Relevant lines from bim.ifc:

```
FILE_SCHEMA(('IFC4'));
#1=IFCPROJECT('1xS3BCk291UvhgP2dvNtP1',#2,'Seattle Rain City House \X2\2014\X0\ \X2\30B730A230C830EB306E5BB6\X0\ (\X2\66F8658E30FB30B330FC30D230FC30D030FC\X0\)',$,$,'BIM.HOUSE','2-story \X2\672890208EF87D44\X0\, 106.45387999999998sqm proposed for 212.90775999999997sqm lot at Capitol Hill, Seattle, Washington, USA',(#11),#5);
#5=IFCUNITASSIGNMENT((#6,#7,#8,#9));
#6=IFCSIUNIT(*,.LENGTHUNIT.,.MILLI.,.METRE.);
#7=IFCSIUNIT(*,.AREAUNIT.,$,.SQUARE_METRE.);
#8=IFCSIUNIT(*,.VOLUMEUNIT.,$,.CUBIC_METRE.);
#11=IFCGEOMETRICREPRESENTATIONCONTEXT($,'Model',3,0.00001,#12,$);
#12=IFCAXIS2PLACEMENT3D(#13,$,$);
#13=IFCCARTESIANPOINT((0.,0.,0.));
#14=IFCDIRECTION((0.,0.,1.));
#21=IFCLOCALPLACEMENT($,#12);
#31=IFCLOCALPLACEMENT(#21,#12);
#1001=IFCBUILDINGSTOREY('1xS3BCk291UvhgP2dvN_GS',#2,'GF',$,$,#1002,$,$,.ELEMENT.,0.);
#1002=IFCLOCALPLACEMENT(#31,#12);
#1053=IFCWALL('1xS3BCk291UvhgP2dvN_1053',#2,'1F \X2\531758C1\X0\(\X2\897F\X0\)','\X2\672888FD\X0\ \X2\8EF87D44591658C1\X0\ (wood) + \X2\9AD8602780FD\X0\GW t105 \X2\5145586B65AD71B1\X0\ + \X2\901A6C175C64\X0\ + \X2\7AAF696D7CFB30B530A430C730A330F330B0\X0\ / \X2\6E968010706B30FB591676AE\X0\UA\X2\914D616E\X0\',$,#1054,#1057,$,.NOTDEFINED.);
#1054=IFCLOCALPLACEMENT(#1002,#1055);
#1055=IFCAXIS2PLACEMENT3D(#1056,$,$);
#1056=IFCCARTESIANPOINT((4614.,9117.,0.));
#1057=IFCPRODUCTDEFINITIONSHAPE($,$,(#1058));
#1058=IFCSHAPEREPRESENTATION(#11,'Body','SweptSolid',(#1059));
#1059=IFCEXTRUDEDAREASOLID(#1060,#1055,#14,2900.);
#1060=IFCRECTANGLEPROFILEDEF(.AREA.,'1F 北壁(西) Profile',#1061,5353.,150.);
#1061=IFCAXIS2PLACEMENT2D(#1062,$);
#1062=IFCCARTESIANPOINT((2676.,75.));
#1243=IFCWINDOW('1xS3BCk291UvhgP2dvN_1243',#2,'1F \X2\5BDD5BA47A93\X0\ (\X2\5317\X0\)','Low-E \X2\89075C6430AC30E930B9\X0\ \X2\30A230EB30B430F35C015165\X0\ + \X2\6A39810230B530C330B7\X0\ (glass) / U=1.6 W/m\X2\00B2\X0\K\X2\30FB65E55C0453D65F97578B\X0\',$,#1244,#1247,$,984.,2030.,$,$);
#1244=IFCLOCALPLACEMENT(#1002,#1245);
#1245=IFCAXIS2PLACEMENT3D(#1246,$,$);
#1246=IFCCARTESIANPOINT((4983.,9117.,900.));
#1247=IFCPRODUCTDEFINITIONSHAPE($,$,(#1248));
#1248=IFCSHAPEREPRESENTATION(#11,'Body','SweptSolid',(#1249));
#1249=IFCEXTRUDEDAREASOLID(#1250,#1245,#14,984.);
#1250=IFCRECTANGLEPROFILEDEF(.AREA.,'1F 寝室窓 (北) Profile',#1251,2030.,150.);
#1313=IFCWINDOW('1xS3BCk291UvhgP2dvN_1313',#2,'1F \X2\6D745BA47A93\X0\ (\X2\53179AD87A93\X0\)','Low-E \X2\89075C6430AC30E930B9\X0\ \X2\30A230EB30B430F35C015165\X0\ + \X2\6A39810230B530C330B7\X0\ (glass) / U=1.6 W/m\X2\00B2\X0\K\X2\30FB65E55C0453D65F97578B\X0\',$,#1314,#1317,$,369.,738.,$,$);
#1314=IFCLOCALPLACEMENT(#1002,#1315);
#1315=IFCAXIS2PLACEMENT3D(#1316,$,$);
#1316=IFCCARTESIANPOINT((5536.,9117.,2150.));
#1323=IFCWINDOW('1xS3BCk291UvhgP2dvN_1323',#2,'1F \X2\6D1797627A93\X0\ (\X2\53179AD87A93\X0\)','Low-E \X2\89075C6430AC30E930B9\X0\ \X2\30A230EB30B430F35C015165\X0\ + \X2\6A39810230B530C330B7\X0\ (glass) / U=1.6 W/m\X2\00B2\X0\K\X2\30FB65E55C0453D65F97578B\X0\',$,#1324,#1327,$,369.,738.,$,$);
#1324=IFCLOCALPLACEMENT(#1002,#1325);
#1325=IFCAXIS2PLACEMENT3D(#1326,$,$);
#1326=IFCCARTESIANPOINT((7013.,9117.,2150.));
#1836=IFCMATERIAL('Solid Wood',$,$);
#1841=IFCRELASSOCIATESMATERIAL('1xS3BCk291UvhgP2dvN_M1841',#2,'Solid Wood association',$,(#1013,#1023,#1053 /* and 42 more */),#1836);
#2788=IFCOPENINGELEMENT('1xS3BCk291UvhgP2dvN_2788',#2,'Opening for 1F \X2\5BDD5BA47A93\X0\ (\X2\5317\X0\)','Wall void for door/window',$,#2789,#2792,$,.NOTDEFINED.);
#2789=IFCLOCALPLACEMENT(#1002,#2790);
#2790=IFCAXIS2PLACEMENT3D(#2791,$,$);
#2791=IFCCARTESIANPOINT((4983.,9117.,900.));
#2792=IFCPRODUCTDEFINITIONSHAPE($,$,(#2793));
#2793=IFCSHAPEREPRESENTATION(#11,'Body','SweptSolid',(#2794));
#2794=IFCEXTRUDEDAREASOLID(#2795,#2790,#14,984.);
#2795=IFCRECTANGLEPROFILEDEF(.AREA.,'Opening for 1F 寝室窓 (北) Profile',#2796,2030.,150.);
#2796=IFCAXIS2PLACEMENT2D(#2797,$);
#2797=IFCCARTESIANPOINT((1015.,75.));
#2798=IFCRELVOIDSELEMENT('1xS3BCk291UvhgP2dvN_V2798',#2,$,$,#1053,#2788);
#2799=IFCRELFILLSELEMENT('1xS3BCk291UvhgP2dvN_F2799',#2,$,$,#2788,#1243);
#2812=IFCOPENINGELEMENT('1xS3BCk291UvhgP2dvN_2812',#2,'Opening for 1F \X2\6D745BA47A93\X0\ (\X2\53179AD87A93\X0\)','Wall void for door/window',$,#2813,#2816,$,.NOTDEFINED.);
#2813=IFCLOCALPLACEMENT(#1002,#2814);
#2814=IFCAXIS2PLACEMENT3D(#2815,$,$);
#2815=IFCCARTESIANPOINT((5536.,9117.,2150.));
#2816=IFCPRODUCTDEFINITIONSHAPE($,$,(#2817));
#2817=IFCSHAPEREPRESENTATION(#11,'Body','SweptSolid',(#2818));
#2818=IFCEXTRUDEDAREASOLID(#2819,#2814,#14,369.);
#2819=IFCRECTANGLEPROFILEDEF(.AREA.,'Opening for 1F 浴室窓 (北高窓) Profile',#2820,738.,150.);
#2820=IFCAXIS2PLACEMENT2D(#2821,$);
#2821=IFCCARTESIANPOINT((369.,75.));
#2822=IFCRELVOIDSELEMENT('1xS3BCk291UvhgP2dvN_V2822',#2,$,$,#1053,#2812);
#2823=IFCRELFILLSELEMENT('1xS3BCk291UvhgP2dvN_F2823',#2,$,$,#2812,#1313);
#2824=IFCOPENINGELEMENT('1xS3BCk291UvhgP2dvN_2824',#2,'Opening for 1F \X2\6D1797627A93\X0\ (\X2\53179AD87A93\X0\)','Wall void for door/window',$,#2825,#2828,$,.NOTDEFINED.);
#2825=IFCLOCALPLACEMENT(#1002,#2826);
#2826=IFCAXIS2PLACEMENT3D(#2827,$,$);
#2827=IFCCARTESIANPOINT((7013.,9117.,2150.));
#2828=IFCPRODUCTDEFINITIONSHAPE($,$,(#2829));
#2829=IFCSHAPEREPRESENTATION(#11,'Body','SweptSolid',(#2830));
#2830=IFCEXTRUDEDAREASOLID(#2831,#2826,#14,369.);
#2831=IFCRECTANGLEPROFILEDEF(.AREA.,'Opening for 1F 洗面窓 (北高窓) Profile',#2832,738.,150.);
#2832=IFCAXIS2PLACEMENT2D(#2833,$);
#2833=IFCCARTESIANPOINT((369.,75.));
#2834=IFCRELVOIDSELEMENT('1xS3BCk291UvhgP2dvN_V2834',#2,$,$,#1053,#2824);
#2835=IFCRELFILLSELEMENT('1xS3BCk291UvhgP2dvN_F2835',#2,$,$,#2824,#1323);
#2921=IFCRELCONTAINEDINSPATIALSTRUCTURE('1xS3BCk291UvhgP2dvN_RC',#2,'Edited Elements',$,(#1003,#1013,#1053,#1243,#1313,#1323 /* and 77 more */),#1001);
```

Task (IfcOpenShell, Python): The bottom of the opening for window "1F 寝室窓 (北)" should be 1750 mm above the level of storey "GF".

```python
import numpy as np
import ifcopenshell
import ifcopenshell.api.geometry
import ifcopenshell.geom
import ifcopenshell.util.element
import ifcopenshell.util.placement
import ifcopenshell.util.shape
import ifcopenshell.util.unit

model = ifcopenshell.open("bim.ifc")
unit_scale = ifcopenshell.util.unit.calculate_unit_scale(model)

window = model.by_guid("1xS3BCk291UvhgP2dvN_1243")
opening = window.FillsVoids[0].RelatingOpeningElement
storey = ifcopenshell.util.element.get_container(window, ifc_class="IfcBuildingStorey")
level = ifcopenshell.util.placement.get_local_placement(storey.ObjectPlacement)[2, 3]

# The opening's origin need not be at the sill, so measure its lowest point.
shape = ifcopenshell.geom.create_shape(ifcopenshell.geom.settings(), opening)
bottom = ifcopenshell.util.shape.get_shape_bottom_elevation(shape, shape.geometry) / unit_scale
dz = level + 1750.0 - bottom

shift = np.array([0.0, 0.0, dz])
# The window is not placed relative to its opening, so move both.
for product in (opening, window):
    matrix = ifcopenshell.util.placement.get_local_placement(product.ObjectPlacement)
    matrix[:3, 3] += shift
    ifcopenshell.api.geometry.edit_object_placement(model, product=product, matrix=matrix, is_si=False)

print(f"moved by {dz * unit_scale:+.3f} m")

model.write("bim-out.ifc")
```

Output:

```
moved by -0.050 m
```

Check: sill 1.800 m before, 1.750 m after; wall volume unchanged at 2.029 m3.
